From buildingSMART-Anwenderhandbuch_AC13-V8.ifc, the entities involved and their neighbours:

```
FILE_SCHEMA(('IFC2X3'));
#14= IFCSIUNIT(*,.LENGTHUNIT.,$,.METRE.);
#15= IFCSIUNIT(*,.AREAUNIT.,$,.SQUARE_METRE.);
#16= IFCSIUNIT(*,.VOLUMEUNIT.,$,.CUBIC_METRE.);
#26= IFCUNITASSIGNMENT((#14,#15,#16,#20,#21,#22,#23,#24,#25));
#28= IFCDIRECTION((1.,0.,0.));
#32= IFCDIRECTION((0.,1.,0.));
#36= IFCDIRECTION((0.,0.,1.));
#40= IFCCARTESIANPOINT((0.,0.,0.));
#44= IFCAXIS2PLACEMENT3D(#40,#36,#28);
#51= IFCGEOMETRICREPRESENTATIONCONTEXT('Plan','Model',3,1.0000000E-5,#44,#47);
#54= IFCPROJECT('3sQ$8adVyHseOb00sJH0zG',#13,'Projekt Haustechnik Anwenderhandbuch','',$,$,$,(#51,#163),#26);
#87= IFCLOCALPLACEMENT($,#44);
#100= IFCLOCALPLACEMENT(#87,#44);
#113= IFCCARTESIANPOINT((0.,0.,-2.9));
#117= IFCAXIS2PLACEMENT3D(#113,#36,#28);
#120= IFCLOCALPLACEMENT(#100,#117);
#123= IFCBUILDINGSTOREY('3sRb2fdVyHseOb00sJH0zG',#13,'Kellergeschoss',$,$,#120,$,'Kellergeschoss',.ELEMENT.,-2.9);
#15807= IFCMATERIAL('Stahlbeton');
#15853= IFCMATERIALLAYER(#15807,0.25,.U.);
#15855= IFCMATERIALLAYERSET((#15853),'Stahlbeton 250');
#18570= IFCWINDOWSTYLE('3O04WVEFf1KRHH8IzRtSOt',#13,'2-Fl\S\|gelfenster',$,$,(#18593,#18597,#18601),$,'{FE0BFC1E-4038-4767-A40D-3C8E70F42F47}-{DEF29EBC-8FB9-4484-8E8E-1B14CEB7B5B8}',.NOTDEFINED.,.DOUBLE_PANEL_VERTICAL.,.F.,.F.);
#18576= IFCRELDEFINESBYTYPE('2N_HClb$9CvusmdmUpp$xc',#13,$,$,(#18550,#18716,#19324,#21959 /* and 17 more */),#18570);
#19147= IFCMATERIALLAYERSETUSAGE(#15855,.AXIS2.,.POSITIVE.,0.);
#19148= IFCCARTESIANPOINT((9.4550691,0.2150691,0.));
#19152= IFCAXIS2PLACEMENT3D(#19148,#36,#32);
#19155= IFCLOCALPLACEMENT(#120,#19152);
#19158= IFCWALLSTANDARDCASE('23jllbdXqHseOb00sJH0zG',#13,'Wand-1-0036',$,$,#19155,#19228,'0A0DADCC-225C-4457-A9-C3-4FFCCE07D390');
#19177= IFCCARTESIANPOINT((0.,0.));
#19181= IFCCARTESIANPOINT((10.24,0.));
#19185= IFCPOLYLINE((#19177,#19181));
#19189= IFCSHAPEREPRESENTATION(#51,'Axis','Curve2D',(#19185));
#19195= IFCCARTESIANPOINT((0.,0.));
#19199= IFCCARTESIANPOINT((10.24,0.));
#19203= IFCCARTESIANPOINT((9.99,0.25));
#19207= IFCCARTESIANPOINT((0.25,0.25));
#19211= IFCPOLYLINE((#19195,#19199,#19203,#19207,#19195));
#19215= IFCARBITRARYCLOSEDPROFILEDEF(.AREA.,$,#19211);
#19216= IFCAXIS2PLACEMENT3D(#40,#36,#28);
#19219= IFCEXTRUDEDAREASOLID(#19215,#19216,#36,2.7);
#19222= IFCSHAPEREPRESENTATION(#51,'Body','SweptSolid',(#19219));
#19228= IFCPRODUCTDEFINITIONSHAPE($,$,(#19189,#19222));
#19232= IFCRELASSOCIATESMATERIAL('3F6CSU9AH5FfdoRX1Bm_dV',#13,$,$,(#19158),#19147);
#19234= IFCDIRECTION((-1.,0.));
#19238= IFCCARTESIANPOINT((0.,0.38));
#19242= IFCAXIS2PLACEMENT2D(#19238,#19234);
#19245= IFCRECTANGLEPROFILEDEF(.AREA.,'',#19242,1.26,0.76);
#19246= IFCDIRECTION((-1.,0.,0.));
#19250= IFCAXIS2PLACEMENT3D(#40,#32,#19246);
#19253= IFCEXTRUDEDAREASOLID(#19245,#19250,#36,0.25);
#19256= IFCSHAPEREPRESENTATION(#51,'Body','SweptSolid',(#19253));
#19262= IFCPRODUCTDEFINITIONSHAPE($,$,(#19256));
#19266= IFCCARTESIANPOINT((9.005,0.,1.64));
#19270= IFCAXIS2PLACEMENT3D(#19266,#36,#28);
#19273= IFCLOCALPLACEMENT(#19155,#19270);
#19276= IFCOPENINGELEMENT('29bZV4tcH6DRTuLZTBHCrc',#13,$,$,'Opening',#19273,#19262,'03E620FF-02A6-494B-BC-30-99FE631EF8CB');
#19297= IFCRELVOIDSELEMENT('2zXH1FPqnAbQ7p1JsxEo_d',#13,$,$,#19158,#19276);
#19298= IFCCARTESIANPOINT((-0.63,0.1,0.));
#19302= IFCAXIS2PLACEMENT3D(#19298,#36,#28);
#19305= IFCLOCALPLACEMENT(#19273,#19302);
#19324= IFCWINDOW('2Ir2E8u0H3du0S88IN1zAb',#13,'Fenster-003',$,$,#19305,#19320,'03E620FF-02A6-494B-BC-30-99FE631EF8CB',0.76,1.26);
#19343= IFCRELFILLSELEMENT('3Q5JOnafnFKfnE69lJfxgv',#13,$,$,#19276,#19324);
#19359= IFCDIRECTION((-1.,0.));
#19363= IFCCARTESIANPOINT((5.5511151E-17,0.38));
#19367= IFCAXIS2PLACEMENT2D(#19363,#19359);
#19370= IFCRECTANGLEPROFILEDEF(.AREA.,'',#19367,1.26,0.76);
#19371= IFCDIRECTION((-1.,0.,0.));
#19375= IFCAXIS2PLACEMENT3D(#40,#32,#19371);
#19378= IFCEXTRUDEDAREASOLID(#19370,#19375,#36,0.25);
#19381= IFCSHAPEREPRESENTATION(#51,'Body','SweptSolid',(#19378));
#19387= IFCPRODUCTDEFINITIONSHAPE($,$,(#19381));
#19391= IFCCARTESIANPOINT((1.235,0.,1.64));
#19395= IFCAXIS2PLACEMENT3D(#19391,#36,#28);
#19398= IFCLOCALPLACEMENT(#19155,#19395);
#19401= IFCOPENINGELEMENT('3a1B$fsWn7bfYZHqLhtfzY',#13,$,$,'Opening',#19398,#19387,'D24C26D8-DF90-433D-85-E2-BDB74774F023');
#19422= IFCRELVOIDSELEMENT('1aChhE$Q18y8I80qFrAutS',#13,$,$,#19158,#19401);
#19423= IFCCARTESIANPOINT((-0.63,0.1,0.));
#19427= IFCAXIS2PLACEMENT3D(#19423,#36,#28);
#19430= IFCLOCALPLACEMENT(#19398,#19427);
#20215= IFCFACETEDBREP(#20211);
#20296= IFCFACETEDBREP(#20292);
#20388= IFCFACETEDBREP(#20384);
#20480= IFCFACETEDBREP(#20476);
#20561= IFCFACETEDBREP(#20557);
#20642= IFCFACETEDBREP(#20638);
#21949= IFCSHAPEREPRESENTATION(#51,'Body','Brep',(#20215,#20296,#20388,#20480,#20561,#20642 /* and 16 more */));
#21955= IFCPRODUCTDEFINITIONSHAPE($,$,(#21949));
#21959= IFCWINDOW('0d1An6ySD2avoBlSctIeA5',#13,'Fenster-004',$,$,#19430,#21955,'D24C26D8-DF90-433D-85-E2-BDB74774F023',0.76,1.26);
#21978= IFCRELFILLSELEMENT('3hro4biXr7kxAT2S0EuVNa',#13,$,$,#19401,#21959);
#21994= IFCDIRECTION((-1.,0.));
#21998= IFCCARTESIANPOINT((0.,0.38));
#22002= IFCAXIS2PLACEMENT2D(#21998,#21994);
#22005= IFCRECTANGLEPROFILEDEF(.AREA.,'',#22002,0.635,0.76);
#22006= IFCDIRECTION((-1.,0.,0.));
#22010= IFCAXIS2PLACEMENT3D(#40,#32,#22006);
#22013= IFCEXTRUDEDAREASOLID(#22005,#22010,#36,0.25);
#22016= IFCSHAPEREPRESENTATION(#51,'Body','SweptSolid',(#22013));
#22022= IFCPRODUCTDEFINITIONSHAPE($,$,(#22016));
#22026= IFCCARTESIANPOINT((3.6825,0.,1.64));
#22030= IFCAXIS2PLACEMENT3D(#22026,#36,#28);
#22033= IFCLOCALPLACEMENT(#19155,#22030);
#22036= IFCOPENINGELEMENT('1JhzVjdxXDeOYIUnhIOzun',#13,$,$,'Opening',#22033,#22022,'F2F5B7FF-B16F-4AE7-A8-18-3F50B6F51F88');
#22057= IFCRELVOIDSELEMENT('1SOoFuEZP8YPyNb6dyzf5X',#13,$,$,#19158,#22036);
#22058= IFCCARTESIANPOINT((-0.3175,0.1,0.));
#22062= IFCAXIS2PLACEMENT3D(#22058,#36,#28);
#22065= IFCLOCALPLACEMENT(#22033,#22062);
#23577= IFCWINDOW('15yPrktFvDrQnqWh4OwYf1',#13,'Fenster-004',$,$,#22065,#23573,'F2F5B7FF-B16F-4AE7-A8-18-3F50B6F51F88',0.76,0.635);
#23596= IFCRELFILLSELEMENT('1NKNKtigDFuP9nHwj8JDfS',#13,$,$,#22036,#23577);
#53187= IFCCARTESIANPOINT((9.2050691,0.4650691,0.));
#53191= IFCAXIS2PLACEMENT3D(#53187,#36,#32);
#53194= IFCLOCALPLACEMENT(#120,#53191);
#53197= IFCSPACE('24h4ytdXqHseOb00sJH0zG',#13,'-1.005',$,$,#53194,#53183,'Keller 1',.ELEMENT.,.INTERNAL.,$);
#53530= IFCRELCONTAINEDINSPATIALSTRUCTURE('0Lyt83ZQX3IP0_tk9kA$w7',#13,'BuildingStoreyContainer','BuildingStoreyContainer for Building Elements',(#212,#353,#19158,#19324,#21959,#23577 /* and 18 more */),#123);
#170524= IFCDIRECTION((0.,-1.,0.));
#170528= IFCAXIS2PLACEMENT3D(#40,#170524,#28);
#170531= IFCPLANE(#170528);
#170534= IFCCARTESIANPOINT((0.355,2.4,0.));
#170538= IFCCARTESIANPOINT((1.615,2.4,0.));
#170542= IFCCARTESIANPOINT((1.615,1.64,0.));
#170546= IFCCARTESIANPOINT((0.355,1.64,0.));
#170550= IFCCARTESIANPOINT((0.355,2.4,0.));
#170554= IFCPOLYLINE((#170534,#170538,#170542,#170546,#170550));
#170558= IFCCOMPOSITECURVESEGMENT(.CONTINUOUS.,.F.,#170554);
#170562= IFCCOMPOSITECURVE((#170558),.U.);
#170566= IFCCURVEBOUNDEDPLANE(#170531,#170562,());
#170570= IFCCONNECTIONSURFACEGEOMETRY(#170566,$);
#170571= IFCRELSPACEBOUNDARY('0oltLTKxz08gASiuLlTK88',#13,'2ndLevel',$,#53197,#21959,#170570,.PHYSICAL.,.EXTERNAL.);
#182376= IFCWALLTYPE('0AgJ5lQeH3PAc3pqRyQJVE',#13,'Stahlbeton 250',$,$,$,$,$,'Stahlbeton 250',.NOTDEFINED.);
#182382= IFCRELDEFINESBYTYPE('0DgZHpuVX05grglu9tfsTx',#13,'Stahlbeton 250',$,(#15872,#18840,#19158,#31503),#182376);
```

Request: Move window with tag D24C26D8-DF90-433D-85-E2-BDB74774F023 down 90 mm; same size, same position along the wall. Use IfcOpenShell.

```python
import numpy as np
import ifcopenshell
import ifcopenshell.api.geometry
import ifcopenshell.util.placement
import ifcopenshell.util.unit

model = ifcopenshell.open("buildingSMART-Anwenderhandbuch_AC13-V8.ifc")
unit_scale = ifcopenshell.util.unit.calculate_unit_scale(model)

window = model.by_id(21959)
opening = window.FillsVoids[0].RelatingOpeningElement
dz = -0.09

shift = np.array([0.0, 0.0, dz])
# The window is placed relative to its opening, so it follows when the opening moves.
matrix = ifcopenshell.util.placement.get_local_placement(opening.ObjectPlacement)
matrix[:3, 3] += shift
ifcopenshell.api.geometry.edit_object_placement(
    model, product=opening, matrix=matrix, is_si=False, should_transform_children=True
)

# Space boundary surfaces are stored in each space's coordinates; move them too.
for rel in window.ProvidesBoundaries:
    if not rel.ConnectionGeometry:
        continue
    surface = rel.ConnectionGeometry.SurfaceOnRelatingElement.BasisSurface
    space_matrix = ifcopenshell.util.placement.get_local_placement(rel.RelatingSpace.ObjectPlacement)
    point = np.array(surface.Position.Location.Coordinates) + space_matrix[:3, :3].T @ shift
    surface.Position = model.createIfcAxis2Placement3D(
        model.createIfcCartesianPoint(point.tolist()), surface.Position.Axis, surface.Position.RefDirection
    )

print(f"moved by {dz * unit_scale:+.3f} m")

model.write("buildingSMART-Anwenderhandbuch_AC13-V8-out.ifc")
```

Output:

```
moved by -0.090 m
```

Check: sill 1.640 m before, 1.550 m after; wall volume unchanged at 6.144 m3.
